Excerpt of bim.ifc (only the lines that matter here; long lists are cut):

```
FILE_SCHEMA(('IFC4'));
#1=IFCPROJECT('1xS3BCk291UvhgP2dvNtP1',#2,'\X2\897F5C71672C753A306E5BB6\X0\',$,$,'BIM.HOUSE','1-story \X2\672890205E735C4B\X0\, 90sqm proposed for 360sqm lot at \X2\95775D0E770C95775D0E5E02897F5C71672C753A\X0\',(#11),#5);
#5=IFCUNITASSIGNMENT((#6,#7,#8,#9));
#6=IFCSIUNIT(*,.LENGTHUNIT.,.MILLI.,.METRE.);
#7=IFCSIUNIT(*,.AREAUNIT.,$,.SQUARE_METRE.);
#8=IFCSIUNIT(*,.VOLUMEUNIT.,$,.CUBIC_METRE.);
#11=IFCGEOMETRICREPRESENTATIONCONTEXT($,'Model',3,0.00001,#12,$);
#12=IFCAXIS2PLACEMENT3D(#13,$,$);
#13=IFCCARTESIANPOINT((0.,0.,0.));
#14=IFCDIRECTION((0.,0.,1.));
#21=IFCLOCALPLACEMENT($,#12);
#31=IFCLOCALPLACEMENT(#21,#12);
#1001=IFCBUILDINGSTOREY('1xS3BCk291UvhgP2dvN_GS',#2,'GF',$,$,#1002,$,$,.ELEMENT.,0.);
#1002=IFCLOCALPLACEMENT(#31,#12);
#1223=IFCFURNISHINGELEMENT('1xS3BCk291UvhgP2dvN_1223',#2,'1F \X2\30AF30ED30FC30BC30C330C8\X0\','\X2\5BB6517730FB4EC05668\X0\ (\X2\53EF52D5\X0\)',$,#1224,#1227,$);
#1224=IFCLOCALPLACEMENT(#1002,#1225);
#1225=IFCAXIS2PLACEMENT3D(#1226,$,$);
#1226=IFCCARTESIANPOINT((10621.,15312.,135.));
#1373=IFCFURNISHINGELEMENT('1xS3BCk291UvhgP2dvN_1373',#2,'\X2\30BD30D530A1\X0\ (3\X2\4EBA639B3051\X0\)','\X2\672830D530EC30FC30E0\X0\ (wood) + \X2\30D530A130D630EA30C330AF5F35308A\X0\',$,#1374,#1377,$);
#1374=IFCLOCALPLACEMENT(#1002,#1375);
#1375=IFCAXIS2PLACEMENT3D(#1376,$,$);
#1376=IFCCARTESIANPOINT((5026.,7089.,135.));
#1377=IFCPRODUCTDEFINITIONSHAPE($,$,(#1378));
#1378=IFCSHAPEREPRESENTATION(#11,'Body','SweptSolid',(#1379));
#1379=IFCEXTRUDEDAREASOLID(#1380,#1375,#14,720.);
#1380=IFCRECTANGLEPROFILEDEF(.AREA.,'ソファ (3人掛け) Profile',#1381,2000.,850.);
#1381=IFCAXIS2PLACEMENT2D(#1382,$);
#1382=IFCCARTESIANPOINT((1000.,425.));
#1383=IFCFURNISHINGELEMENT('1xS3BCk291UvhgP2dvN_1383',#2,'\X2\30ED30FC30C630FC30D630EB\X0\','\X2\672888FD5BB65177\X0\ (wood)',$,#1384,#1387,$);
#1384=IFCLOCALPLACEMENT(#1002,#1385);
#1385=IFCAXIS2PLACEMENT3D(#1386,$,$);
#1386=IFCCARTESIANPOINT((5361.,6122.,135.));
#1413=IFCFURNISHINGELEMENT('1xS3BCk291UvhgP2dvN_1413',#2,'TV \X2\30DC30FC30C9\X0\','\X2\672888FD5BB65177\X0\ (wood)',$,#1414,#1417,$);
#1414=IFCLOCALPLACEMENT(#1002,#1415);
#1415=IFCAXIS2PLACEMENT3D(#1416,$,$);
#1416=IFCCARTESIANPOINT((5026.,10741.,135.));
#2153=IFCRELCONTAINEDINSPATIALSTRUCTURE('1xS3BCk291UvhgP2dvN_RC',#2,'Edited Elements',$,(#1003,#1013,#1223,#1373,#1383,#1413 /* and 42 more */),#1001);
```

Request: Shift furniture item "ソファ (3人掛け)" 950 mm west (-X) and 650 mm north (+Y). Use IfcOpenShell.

```python
import ifcopenshell
import ifcopenshell.api.geometry
import ifcopenshell.util.placement

model = ifcopenshell.open("bim.ifc")

item = model.by_id(1373)
matrix = ifcopenshell.util.placement.get_local_placement(item.ObjectPlacement)
matrix[0, 3] -= 950.0
matrix[1, 3] += 650.0
ifcopenshell.api.geometry.edit_object_placement(model, product=item, matrix=matrix, is_si=False)

print(ifcopenshell.util.placement.get_local_placement(item.ObjectPlacement).round(3) + 0.0)

model.write("bim_rev.ifc")
```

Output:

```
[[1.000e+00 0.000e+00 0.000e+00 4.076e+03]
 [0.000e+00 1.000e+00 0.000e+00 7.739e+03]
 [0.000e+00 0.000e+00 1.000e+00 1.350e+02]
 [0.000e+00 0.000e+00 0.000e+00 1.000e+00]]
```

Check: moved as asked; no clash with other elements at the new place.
